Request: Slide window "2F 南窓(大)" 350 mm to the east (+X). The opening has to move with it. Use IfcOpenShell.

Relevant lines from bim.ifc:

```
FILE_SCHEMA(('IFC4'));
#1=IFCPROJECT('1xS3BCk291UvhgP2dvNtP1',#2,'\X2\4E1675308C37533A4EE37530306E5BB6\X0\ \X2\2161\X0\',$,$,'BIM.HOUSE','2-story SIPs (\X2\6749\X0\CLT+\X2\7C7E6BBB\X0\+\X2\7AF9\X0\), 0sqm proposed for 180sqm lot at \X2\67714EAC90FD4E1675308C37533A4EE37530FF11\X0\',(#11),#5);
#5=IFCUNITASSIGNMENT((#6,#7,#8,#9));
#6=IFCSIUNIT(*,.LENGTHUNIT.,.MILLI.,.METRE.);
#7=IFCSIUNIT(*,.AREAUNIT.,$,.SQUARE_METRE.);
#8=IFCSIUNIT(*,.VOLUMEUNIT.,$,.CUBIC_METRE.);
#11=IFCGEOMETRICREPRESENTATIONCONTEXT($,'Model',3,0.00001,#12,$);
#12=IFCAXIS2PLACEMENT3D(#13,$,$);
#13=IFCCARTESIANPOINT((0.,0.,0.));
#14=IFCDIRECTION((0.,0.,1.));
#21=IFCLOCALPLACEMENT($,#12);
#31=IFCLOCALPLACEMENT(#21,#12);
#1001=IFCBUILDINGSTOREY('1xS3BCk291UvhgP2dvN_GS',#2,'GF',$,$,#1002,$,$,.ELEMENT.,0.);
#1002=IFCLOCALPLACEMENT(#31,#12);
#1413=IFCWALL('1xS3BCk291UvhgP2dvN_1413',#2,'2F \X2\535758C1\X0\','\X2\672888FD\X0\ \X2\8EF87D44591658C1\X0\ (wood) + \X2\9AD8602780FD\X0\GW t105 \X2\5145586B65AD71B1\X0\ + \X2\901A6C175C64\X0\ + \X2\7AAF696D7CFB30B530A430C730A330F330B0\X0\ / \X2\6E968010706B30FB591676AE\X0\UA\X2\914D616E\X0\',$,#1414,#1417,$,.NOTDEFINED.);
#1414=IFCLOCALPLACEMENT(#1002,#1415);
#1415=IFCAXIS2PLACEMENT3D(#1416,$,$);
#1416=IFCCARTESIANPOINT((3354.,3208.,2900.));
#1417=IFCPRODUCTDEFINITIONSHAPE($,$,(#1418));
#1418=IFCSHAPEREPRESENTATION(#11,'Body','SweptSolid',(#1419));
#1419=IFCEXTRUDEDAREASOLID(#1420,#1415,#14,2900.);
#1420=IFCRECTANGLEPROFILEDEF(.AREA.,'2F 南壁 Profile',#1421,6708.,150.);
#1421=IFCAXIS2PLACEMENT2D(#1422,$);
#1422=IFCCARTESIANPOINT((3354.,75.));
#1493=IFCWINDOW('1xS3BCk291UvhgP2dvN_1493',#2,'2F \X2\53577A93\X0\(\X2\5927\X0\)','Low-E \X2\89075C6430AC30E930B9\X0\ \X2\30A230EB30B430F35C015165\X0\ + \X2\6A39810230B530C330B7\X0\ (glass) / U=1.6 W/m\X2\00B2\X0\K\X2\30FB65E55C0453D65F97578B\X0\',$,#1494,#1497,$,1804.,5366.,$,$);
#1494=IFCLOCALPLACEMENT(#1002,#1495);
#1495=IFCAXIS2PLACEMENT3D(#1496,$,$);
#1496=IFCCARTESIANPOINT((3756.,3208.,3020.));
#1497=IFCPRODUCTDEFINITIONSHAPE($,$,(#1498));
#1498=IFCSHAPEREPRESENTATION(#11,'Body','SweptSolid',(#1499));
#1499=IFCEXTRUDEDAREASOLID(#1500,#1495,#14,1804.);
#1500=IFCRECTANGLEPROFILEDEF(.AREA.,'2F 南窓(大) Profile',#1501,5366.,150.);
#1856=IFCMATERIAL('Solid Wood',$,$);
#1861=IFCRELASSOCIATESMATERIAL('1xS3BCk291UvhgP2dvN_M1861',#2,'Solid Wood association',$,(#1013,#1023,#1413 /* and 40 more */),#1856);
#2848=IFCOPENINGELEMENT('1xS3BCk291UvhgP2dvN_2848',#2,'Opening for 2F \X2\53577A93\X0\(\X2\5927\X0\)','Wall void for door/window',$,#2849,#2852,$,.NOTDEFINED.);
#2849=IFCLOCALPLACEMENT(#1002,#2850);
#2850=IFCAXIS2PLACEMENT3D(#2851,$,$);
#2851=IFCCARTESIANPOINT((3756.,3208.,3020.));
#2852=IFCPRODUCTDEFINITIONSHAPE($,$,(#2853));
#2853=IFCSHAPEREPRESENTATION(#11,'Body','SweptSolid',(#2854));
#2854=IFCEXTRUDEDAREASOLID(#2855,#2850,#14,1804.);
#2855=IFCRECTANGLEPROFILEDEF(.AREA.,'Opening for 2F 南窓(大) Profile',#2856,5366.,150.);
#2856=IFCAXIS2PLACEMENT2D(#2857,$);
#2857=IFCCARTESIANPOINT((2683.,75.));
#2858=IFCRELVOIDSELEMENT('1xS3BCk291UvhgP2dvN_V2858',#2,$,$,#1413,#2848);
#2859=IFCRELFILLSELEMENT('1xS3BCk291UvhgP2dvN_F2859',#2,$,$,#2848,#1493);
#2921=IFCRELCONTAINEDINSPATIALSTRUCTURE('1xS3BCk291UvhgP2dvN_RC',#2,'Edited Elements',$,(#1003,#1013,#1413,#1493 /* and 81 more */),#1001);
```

```python
import ifcopenshell
import ifcopenshell.api.geometry
import ifcopenshell.util.placement

model = ifcopenshell.open("bim.ifc")

window = model.by_guid("1xS3BCk291UvhgP2dvN_1493")
opening = window.FillsVoids[0].RelatingOpeningElement
wall = opening.VoidsElements[0].RelatingBuildingElement

wall_matrix = ifcopenshell.util.placement.get_local_placement(wall.ObjectPlacement)
shift = wall_matrix[:3, 0] * 350.0
before = ifcopenshell.util.placement.get_local_placement(window.ObjectPlacement)[:3, 3].copy()

# The window is not placed relative to its opening, so move both.
for product in (opening, window):
    matrix = ifcopenshell.util.placement.get_local_placement(product.ObjectPlacement)
    matrix[:3, 3] += shift
    ifcopenshell.api.geometry.edit_object_placement(model, product=product, matrix=matrix, is_si=False)

after = ifcopenshell.util.placement.get_local_placement(window.ObjectPlacement)[:3, 3]
print("window moved by", (after - before).round(3) + 0.0)

model.write("bim_rev.ifc")
```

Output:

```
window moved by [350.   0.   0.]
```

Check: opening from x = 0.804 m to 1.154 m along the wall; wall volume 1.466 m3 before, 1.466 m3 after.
